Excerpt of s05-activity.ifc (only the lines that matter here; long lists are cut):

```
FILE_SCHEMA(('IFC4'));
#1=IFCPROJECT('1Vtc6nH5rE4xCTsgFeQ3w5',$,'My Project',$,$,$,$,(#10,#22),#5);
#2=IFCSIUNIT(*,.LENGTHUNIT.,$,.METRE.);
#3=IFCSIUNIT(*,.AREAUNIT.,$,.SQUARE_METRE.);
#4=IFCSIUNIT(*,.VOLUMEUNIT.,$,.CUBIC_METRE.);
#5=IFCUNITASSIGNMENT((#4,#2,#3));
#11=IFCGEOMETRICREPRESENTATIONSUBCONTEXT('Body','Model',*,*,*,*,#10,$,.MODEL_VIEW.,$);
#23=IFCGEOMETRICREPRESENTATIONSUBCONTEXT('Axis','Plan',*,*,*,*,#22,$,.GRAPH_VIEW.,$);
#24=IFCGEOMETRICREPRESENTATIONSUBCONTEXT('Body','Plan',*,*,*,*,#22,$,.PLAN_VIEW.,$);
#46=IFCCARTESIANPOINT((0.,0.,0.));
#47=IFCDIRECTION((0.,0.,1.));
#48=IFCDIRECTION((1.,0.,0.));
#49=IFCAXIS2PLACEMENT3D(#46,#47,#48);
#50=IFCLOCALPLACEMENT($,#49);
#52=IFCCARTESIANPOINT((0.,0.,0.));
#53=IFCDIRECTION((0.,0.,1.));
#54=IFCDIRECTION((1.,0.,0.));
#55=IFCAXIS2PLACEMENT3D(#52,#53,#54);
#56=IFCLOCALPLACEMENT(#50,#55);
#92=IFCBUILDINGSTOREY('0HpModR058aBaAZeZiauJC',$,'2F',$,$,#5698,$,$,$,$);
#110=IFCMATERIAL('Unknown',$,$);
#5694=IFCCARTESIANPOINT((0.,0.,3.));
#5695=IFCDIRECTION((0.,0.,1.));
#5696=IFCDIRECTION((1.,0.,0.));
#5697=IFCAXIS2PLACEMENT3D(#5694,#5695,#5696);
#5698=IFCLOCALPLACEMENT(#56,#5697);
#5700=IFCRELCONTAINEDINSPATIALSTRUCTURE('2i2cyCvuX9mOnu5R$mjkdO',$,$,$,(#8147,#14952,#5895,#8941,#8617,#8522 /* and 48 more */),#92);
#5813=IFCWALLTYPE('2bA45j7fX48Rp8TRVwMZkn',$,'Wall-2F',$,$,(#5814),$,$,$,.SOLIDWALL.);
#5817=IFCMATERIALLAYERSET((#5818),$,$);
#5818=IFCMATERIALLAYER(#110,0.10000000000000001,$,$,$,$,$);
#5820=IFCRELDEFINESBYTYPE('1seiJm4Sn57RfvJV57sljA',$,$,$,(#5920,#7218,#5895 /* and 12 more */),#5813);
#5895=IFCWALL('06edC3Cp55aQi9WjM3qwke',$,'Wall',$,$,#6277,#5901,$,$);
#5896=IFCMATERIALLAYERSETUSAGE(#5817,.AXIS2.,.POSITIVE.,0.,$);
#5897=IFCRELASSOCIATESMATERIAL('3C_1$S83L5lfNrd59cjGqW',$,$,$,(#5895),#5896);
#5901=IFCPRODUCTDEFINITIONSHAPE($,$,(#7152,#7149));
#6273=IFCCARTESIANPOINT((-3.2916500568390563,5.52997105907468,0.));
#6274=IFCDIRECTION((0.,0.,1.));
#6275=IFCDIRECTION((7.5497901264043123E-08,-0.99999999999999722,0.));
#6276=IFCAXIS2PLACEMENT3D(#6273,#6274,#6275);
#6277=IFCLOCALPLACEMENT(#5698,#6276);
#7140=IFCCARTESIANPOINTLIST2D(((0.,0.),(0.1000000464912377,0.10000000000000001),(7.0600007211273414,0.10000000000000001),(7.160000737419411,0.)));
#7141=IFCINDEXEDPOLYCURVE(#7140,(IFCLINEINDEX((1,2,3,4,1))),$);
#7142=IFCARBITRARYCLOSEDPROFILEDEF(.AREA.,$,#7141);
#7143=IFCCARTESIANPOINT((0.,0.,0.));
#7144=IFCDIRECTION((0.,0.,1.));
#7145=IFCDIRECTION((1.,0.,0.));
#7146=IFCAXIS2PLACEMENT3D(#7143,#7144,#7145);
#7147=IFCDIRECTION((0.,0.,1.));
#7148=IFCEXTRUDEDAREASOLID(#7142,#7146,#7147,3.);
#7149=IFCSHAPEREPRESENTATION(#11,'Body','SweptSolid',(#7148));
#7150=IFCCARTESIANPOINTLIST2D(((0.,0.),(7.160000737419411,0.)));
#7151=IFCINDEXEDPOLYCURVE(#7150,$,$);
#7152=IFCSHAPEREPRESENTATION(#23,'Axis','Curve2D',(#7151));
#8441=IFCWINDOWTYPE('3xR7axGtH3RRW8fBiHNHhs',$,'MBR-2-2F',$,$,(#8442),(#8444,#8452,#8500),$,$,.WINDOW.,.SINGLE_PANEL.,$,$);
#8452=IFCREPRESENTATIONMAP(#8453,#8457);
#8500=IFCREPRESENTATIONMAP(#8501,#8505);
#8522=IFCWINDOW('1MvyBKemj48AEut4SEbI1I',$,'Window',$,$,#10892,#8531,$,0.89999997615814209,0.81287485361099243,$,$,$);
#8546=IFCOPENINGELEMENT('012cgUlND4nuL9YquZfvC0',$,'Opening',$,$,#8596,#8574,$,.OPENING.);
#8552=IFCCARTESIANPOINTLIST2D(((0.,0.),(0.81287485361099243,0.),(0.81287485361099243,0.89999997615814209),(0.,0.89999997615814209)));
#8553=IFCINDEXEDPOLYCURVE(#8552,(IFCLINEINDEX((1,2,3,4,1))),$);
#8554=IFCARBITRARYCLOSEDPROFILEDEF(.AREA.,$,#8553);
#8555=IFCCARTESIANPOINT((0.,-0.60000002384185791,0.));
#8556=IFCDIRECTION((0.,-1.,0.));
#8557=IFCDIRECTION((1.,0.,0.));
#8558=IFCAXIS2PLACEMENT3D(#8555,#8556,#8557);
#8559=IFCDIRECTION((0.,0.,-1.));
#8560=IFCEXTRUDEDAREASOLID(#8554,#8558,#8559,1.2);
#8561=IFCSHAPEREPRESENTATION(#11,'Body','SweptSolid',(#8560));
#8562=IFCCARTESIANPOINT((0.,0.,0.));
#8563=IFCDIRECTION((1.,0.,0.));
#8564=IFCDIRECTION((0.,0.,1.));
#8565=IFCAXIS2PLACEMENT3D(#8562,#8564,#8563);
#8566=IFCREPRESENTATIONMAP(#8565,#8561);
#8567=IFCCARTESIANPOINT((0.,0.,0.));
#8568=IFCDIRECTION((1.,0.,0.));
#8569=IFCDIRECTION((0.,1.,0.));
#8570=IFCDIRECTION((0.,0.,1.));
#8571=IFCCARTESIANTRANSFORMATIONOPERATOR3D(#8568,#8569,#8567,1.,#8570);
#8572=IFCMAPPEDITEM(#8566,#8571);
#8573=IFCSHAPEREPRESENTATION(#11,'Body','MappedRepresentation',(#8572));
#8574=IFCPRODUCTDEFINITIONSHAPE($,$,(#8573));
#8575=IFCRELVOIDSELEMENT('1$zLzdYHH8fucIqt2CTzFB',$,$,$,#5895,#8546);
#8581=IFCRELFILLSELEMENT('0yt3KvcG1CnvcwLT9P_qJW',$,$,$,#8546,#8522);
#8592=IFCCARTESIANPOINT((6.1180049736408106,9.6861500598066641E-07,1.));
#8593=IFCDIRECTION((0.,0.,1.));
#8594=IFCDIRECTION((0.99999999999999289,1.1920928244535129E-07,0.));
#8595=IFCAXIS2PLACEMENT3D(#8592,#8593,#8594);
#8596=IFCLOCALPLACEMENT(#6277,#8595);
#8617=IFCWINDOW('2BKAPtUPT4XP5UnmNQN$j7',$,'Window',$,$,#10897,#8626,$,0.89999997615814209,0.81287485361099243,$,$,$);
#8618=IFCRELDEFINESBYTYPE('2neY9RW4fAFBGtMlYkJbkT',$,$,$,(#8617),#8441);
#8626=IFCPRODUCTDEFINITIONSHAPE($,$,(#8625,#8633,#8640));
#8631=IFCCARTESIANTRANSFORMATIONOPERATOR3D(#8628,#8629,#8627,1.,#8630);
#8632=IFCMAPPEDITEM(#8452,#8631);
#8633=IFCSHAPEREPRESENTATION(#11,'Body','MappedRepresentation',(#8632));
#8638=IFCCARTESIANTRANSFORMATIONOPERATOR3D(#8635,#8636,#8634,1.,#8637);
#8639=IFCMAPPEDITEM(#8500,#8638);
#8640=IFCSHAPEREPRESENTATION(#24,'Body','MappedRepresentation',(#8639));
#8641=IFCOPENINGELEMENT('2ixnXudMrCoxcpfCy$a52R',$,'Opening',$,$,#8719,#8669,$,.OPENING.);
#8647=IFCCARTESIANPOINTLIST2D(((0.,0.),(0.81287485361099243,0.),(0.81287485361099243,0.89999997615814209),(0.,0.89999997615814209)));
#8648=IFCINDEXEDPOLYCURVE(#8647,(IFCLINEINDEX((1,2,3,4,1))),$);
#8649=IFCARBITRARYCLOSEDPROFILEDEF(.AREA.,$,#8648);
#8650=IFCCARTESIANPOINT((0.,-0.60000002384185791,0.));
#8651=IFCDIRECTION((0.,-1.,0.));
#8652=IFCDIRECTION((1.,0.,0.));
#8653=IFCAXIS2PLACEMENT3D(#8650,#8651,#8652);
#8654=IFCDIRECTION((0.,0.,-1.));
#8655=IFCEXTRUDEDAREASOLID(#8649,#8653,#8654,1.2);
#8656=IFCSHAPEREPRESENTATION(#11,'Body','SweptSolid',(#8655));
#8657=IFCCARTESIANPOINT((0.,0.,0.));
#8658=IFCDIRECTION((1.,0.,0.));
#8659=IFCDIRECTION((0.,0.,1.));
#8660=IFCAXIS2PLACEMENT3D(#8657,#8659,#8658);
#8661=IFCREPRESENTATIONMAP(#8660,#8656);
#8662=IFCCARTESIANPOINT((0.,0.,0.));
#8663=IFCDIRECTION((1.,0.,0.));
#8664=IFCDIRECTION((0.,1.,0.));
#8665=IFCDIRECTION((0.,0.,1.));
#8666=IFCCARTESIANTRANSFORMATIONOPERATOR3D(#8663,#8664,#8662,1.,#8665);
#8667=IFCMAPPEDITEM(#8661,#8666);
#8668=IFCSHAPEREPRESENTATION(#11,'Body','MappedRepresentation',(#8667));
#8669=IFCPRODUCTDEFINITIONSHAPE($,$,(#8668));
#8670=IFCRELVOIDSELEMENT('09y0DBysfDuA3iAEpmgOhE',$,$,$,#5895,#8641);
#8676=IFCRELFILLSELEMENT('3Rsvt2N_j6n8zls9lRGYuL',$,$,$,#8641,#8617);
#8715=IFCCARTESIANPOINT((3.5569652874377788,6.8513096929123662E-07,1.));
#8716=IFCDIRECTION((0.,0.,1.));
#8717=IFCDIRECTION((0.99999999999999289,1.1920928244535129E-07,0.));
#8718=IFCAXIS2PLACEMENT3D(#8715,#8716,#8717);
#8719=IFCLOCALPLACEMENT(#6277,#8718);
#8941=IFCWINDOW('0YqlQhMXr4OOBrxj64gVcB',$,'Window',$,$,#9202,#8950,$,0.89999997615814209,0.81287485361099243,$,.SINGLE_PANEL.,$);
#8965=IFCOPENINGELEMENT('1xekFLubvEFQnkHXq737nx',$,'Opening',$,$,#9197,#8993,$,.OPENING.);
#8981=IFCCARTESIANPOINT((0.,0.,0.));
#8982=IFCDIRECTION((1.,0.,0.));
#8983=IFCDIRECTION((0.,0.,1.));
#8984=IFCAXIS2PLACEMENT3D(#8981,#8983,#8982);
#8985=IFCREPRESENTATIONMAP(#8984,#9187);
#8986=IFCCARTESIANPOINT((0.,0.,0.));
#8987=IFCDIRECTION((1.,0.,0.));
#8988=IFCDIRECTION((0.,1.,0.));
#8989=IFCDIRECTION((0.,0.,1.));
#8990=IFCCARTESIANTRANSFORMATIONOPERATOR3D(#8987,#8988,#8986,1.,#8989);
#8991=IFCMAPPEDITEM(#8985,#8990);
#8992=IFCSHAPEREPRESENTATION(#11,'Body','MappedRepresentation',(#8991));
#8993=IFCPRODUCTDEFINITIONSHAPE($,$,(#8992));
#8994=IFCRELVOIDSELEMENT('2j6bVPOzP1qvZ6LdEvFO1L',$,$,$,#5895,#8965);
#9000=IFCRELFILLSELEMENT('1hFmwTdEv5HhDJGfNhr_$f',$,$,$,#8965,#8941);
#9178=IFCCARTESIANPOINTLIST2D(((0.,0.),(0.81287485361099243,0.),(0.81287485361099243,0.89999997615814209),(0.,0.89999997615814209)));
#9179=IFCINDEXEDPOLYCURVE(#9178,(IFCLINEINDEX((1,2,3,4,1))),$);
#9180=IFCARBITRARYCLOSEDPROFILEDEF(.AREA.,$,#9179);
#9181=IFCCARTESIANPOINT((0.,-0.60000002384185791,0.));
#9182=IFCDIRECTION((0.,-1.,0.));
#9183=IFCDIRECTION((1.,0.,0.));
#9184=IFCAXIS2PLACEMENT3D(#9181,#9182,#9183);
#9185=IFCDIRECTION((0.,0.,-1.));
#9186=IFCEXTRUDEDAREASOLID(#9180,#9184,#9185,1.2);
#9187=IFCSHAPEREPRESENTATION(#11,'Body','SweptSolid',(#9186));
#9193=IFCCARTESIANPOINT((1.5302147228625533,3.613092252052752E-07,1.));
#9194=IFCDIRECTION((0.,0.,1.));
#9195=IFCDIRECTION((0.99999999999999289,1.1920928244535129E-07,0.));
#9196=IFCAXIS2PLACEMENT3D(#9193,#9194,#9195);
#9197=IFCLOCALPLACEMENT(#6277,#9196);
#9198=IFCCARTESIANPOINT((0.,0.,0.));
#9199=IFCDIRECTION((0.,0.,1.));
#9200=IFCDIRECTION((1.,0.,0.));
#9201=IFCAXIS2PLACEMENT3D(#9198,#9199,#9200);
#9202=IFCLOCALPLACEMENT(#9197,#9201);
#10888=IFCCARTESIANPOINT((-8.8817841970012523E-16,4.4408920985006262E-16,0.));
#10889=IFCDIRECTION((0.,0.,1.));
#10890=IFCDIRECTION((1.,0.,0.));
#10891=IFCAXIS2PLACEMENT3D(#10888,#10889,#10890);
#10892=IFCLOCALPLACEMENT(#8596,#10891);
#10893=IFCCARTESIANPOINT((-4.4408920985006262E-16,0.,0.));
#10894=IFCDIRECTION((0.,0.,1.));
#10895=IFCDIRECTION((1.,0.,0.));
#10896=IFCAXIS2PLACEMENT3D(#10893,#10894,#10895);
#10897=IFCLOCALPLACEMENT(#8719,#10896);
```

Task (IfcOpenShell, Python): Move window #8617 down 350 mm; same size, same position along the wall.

```python
import numpy as np
import ifcopenshell
import ifcopenshell.api.geometry
import ifcopenshell.util.placement
import ifcopenshell.util.unit

model = ifcopenshell.open("s05-activity.ifc")
unit_scale = ifcopenshell.util.unit.calculate_unit_scale(model)

window = model.by_id(8617)
opening = window.FillsVoids[0].RelatingOpeningElement
dz = -0.35 / unit_scale

shift = np.array([0.0, 0.0, dz])
# The window is placed relative to its opening, so it follows when the opening moves.
matrix = ifcopenshell.util.placement.get_local_placement(opening.ObjectPlacement)
matrix[:3, 3] += shift
ifcopenshell.api.geometry.edit_object_placement(
    model, product=opening, matrix=matrix, is_si=False, should_transform_children=True
)

print(f"moved by {dz * unit_scale:+.3f} m")

model.write("s05-activity_v2.ifc")
```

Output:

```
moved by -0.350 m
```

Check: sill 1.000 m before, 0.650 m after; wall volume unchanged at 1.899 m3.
